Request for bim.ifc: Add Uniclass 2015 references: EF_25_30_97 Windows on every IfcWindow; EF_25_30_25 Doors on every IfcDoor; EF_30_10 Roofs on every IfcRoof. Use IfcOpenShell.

First a look at what the model holds.

```python
import ifcopenshell

model = ifcopenshell.open("bim.ifc")
print(model.schema)
print("classifications:", [c.Name for c in model.by_type("IfcClassification")])
for ifc_class in ("IfcDoor", "IfcRoof", "IfcStair", "IfcWall", "IfcWindow"):
    print(ifc_class, len(model.by_type(ifc_class)))
```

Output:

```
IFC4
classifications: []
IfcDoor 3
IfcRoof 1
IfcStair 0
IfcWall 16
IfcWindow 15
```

```python
import ifcopenshell
import ifcopenshell.api.classification

model = ifcopenshell.open("bim.ifc")

system = ifcopenshell.api.classification.add_classification(model, classification="Uniclass 2015")

codes = {
    "IfcWindow": ("EF_25_30_97", "Windows"),
    "IfcDoor": ("EF_25_30_25", "Doors"),
    "IfcRoof": ("EF_30_10", "Roofs"),
}
for ifc_class, (code, name) in codes.items():
    products = model.by_type(ifc_class)
    ifcopenshell.api.classification.add_reference(
        model, products=products, classification=system, identification=code, name=name
    )
    print(code, len(products))

model.write("bim_v2.ifc")
```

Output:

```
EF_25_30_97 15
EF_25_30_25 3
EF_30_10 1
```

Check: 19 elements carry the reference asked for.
